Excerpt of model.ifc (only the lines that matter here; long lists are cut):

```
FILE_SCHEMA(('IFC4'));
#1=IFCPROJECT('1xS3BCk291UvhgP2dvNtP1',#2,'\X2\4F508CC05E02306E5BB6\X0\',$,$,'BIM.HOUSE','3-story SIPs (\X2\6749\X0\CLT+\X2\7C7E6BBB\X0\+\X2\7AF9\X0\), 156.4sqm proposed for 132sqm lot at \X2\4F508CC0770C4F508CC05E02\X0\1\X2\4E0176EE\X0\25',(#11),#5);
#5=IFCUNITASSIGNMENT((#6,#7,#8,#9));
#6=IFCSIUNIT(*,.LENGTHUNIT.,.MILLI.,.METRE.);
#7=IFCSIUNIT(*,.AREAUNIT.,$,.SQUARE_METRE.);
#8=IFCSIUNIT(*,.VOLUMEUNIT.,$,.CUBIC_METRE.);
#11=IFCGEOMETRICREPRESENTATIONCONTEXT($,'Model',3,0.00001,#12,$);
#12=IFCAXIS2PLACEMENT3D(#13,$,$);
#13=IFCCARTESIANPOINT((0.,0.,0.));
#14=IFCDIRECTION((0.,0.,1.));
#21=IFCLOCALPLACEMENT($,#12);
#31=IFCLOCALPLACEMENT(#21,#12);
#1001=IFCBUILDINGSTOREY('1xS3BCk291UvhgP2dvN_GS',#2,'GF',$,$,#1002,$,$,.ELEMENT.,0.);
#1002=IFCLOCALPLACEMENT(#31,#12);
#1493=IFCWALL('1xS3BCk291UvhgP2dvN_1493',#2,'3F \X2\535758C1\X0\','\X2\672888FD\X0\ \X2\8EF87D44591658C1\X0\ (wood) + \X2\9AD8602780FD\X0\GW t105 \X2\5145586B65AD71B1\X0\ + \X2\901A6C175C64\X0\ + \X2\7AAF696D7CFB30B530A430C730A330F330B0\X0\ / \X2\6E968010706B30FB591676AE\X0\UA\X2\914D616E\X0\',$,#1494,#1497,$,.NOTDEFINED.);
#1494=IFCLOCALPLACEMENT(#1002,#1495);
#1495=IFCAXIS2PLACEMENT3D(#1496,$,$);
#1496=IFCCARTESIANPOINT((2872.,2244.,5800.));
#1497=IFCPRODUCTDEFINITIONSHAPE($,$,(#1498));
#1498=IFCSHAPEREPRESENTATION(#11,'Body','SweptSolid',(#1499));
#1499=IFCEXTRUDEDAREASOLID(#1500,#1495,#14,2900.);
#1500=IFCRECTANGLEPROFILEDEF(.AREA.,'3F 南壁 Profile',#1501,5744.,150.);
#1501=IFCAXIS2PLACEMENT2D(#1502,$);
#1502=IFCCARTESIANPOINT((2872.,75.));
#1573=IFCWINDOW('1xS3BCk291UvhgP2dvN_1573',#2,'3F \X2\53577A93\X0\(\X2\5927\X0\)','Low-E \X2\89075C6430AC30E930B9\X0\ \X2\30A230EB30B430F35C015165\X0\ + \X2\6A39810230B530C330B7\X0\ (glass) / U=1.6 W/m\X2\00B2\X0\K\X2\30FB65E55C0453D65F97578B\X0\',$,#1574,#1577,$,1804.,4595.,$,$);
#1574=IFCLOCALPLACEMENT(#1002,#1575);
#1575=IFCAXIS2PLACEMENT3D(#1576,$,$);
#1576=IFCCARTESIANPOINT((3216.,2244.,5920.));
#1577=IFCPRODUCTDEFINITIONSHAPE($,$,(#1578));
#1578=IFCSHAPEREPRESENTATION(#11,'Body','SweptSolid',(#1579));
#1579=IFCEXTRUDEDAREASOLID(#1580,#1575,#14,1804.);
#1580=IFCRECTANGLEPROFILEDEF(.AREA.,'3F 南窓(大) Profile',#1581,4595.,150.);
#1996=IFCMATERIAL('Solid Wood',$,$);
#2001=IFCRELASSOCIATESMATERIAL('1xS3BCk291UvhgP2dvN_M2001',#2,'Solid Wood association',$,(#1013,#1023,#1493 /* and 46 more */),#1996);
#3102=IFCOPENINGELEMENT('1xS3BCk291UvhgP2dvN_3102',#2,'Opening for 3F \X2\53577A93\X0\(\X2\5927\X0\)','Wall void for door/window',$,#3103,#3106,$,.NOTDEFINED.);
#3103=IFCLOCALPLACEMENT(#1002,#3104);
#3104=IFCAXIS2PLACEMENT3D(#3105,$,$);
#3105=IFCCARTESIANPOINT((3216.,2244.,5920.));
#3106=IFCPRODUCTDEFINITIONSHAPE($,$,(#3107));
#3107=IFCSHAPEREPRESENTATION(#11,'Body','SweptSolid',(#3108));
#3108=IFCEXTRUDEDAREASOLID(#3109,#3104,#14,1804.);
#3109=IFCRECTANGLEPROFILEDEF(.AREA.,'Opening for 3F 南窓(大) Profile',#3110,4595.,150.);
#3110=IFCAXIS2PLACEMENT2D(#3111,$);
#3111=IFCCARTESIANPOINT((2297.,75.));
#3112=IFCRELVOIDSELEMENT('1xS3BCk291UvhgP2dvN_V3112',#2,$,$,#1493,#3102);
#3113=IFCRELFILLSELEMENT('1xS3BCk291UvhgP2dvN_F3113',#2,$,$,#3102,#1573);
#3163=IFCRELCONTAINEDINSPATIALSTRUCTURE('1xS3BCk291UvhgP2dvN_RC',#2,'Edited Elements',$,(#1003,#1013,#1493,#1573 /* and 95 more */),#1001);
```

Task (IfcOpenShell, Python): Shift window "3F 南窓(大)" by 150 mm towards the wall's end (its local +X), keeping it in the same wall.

```python
import ifcopenshell
import ifcopenshell.api.geometry
import ifcopenshell.util.placement

model = ifcopenshell.open("model.ifc")

window = model.by_guid("1xS3BCk291UvhgP2dvN_1573")
opening = window.FillsVoids[0].RelatingOpeningElement
wall = opening.VoidsElements[0].RelatingBuildingElement

wall_matrix = ifcopenshell.util.placement.get_local_placement(wall.ObjectPlacement)
shift = wall_matrix[:3, 0] * 150.0
before = ifcopenshell.util.placement.get_local_placement(window.ObjectPlacement)[:3, 3].copy()

# The window is not placed relative to its opening, so move both.
for product in (opening, window):
    matrix = ifcopenshell.util.placement.get_local_placement(product.ObjectPlacement)
    matrix[:3, 3] += shift
    ifcopenshell.api.geometry.edit_object_placement(model, product=product, matrix=matrix, is_si=False)

after = ifcopenshell.util.placement.get_local_placement(window.ObjectPlacement)[:3, 3]
print("window moved by", (after - before).round(3) + 0.0)

model.write("model_rev.ifc")
```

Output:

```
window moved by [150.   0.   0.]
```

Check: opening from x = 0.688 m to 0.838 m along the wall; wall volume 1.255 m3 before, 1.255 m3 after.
